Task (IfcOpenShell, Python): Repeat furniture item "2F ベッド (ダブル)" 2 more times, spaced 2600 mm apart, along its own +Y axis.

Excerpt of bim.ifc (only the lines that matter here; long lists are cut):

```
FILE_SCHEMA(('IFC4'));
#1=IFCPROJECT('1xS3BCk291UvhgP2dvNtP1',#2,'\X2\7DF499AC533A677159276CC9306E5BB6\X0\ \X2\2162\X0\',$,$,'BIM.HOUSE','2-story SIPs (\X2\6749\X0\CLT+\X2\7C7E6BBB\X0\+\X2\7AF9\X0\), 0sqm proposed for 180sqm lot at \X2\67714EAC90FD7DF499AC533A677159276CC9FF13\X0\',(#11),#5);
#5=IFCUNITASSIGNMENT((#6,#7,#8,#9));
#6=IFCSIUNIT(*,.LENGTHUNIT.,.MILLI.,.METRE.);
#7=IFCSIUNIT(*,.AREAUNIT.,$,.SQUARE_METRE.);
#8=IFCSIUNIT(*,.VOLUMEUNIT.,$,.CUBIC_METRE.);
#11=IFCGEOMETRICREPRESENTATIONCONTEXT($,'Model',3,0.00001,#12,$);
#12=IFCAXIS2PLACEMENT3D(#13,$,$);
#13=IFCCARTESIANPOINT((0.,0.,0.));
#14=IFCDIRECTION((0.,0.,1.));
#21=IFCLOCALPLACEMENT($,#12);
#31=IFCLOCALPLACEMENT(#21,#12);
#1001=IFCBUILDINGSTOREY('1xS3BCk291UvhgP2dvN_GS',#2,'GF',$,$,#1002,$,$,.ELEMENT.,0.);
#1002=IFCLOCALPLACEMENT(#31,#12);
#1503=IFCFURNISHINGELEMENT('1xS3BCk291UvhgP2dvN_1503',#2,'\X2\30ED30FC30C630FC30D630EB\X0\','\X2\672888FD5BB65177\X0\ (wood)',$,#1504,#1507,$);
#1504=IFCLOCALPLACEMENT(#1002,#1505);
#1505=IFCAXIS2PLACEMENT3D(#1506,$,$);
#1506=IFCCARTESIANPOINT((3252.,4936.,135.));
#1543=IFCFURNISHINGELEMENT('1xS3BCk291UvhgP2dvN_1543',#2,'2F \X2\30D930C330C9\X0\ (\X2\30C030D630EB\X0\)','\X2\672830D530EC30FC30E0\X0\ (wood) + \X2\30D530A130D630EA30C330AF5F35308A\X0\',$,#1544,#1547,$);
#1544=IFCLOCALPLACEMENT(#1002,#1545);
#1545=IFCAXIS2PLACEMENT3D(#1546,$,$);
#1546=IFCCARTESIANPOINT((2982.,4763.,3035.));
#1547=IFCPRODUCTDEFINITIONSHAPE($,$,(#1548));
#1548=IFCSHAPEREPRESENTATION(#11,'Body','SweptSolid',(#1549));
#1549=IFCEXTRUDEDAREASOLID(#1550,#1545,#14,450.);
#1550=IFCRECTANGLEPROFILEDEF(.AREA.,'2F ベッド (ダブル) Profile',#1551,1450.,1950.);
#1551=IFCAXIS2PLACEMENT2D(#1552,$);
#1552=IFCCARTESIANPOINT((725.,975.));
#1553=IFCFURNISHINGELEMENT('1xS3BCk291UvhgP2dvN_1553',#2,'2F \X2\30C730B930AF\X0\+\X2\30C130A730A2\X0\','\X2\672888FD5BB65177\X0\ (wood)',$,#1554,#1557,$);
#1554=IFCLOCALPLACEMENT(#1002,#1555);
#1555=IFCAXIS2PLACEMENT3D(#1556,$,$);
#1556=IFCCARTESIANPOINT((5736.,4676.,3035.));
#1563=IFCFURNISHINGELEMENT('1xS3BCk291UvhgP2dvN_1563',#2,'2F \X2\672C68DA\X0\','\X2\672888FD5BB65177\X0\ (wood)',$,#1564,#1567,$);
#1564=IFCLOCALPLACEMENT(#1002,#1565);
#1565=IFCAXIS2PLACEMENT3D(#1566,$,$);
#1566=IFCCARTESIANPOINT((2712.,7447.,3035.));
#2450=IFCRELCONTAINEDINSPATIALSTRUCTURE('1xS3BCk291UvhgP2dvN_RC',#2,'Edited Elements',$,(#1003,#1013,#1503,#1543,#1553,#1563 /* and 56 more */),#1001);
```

```python
import ifcopenshell
import ifcopenshell.api.geometry
import ifcopenshell.api.root
import ifcopenshell.util.element
import ifcopenshell.util.placement
import ifcopenshell.util.unit

model = ifcopenshell.open("bim.ifc")
unit_scale = ifcopenshell.util.unit.calculate_unit_scale(model)


def reuse_history(source, copy):
    """copy_class also copies each property set's owner history, people and application; keep the originals."""
    for rel in copy.IsDefinedBy:
        if rel.is_a("IfcRelDefinesByProperties") and (history := rel.RelatingPropertyDefinition.OwnerHistory):
            rel.RelatingPropertyDefinition.OwnerHistory = source.OwnerHistory
            ifcopenshell.util.element.remove_deep2(model, history)


source = model.by_guid("1xS3BCk291UvhgP2dvN_1543")
base = ifcopenshell.util.placement.get_local_placement(source.ObjectPlacement)
step = base[:3, 1] * 2.6 / unit_scale

for i in range(1, 3):
    copy = ifcopenshell.api.root.copy_class(model, product=source)
    copy.Representation = ifcopenshell.util.element.copy_deep(
        model, source.Representation, exclude=["IfcGeometricRepresentationContext", "IfcRepresentationMap"]
    )
    reuse_history(source, copy)
    matrix = base.copy()
    matrix[:3, 3] += i * step
    print("added at", matrix[:3, 3].round(3) + 0.0)
    ifcopenshell.api.geometry.edit_object_placement(model, product=copy, matrix=matrix, is_si=False)

model.write("bim_edited.ifc")
```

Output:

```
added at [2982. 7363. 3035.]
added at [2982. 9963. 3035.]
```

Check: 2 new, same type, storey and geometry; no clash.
